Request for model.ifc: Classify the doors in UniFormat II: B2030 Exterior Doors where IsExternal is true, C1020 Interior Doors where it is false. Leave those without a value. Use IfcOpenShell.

First a look at what the model holds.

```python
import ifcopenshell
import ifcopenshell.util.element

model = ifcopenshell.open("model.ifc")
print(model.schema)
print("classifications:", [c.Name for c in model.by_type("IfcClassification")])
values = [ifcopenshell.util.element.get_pset(e, "Pset_DoorCommon", "IsExternal") for e in model.by_type("IfcDoor")]
for value in (True, False, None):
    print("IsExternal", value, values.count(value))
```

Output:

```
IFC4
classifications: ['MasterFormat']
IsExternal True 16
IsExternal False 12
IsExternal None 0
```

```python
import ifcopenshell
import ifcopenshell.api.classification
import ifcopenshell.util.element

model = ifcopenshell.open("model.ifc")

system = ifcopenshell.api.classification.add_classification(model, classification="UniFormat II")

doors = model.by_type("IfcDoor")
external = {e: ifcopenshell.util.element.get_pset(e, "Pset_DoorCommon", "IsExternal") for e in doors}
for flag, code, name in ((True, "B2030", "Exterior Doors"), (False, "C1020", "Interior Doors")):
    products = [e for e in doors if external[e] is flag]
    ifcopenshell.api.classification.add_reference(
        model, products=products, classification=system, identification=code, name=name
    )
    print(code, len(products))

model.write("model_edited.ifc")
```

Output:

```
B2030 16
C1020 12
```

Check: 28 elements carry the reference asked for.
